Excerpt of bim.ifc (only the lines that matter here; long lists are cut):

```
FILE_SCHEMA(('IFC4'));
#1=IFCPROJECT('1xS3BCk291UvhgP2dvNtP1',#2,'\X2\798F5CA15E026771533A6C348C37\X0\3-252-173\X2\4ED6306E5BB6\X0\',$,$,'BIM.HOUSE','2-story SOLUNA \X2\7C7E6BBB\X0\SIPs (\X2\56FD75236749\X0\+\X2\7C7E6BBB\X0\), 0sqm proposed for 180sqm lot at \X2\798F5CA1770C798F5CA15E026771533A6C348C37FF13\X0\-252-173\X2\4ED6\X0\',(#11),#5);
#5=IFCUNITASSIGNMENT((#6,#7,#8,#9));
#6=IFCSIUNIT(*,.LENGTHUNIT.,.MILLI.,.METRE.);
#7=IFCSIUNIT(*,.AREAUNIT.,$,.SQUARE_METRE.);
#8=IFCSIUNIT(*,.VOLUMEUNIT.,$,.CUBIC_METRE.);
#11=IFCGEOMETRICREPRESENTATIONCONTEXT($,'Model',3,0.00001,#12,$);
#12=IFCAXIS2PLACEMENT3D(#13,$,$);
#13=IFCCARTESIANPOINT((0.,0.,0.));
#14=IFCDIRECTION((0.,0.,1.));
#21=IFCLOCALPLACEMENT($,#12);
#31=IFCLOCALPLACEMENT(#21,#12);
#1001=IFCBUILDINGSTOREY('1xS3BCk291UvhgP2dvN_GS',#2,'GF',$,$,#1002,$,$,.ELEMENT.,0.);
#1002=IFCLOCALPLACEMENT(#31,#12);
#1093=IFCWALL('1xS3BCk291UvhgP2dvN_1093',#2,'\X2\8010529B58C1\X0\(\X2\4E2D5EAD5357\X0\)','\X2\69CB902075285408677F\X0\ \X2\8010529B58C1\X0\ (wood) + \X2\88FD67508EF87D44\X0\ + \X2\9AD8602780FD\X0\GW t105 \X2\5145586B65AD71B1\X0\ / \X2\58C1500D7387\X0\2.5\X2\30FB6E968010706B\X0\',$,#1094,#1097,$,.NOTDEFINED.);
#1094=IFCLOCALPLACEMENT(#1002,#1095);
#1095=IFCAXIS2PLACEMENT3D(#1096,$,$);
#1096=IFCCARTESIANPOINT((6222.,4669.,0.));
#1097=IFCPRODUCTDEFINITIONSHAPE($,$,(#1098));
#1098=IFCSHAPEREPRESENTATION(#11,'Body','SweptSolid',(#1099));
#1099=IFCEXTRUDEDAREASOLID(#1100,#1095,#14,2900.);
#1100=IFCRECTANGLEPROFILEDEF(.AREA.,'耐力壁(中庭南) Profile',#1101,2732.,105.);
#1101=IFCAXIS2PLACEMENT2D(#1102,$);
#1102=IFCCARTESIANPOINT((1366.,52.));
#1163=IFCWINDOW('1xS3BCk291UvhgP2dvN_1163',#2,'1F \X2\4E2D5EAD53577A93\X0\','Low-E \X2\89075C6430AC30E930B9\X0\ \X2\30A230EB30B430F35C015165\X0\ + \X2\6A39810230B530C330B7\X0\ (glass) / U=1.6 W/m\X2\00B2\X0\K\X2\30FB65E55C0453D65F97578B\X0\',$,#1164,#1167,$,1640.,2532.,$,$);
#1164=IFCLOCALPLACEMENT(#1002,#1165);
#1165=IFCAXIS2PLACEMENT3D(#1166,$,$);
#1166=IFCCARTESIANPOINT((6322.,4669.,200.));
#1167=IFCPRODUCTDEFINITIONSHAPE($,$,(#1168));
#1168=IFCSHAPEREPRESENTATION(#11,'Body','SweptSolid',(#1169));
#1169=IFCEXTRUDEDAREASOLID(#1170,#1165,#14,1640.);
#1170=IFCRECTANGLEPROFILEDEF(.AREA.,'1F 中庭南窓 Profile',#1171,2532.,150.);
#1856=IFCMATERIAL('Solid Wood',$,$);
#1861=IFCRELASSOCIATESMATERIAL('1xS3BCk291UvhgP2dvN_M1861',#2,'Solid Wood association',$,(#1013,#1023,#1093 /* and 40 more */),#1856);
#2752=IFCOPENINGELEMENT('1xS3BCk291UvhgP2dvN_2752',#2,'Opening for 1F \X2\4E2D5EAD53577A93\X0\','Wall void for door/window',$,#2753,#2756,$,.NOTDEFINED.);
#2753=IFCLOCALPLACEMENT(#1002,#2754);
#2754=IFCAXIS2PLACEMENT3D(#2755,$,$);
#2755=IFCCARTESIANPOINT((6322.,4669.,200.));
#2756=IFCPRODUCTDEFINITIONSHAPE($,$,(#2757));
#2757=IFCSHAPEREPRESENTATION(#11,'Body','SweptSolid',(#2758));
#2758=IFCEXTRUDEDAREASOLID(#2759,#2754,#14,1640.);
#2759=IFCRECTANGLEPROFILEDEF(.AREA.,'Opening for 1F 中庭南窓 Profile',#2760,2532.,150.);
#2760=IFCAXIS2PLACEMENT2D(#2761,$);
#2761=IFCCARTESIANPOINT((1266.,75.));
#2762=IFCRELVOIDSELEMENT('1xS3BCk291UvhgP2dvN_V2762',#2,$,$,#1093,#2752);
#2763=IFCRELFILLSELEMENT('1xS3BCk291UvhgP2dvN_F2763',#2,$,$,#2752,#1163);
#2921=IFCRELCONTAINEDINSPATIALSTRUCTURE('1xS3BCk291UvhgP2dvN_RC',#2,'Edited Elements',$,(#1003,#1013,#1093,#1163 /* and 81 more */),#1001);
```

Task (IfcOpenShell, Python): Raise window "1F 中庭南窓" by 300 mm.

```python
import numpy as np
import ifcopenshell
import ifcopenshell.api.geometry
import ifcopenshell.util.placement
import ifcopenshell.util.unit

model = ifcopenshell.open("bim.ifc")
unit_scale = ifcopenshell.util.unit.calculate_unit_scale(model)

window = model.by_id(1163)
opening = window.FillsVoids[0].RelatingOpeningElement
dz = 300.0

shift = np.array([0.0, 0.0, dz])
# The window is not placed relative to its opening, so move both.
for product in (opening, window):
    matrix = ifcopenshell.util.placement.get_local_placement(product.ObjectPlacement)
    matrix[:3, 3] += shift
    ifcopenshell.api.geometry.edit_object_placement(model, product=product, matrix=matrix, is_si=False)

print(f"moved by {dz * unit_scale:+.3f} m")

model.write("bim_updated.ifc")
```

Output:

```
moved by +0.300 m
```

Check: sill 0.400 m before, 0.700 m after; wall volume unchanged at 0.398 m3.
